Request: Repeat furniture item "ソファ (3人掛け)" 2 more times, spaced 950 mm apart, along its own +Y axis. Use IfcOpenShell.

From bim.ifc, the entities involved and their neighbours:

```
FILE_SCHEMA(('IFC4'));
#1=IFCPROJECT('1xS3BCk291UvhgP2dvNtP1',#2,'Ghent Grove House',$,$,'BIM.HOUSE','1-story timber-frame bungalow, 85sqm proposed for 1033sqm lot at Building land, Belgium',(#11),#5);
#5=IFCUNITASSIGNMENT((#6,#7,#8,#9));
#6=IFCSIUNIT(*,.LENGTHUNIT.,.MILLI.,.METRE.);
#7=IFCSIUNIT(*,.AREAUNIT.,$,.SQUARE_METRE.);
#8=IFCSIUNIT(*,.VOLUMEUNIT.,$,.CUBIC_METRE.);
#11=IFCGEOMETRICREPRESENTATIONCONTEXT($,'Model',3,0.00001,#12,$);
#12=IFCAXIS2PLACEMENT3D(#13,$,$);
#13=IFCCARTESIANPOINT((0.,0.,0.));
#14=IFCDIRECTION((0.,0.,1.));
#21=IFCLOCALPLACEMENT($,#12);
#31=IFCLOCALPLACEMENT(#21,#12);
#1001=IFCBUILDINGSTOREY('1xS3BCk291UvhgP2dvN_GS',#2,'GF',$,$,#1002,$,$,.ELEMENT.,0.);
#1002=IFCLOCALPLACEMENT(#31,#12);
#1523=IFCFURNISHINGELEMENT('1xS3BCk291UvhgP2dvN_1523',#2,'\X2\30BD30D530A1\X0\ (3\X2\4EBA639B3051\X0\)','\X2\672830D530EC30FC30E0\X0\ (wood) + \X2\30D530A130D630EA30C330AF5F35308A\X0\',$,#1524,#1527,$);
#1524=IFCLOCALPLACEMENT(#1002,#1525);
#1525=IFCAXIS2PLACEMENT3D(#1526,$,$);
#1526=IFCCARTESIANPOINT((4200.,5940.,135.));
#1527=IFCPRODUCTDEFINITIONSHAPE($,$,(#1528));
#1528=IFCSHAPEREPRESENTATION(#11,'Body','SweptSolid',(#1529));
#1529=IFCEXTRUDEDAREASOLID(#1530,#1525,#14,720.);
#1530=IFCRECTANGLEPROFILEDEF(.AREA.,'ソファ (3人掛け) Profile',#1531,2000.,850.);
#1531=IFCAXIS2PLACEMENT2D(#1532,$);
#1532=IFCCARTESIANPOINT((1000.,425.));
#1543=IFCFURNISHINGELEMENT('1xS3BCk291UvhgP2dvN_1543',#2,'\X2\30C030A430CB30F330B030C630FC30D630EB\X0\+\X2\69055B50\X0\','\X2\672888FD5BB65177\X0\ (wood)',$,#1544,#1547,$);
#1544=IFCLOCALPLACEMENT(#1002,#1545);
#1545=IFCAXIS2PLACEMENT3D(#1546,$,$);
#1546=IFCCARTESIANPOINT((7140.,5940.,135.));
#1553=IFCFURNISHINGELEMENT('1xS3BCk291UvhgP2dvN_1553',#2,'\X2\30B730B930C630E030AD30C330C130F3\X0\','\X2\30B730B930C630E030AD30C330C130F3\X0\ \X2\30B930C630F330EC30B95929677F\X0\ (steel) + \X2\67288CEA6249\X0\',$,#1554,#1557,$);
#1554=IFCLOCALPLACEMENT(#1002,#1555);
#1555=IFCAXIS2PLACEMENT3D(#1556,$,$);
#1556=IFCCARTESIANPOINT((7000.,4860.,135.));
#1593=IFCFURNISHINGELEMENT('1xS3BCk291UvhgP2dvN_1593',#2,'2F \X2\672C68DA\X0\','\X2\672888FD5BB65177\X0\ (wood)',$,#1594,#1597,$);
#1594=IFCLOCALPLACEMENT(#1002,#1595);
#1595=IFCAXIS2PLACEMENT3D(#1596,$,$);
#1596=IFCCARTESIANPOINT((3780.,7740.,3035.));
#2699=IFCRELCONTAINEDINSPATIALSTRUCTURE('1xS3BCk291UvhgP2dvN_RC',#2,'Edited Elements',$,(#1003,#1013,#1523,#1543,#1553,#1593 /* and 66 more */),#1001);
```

```python
import ifcopenshell
import ifcopenshell.api.geometry
import ifcopenshell.api.root
import ifcopenshell.util.element
import ifcopenshell.util.placement
import ifcopenshell.util.unit

model = ifcopenshell.open("bim.ifc")
unit_scale = ifcopenshell.util.unit.calculate_unit_scale(model)


def reuse_history(source, copy):
    """copy_class also copies each property set's owner history, people and application; keep the originals."""
    for rel in copy.IsDefinedBy:
        if rel.is_a("IfcRelDefinesByProperties") and (history := rel.RelatingPropertyDefinition.OwnerHistory):
            rel.RelatingPropertyDefinition.OwnerHistory = source.OwnerHistory
            ifcopenshell.util.element.remove_deep2(model, history)


source = model.by_guid("1xS3BCk291UvhgP2dvN_1523")
base = ifcopenshell.util.placement.get_local_placement(source.ObjectPlacement)
step = base[:3, 1] * 0.95 / unit_scale

for i in range(1, 3):
    copy = ifcopenshell.api.root.copy_class(model, product=source)
    copy.Representation = ifcopenshell.util.element.copy_deep(
        model, source.Representation, exclude=["IfcGeometricRepresentationContext", "IfcRepresentationMap"]
    )
    reuse_history(source, copy)
    matrix = base.copy()
    matrix[:3, 3] += i * step
    print("added at", matrix[:3, 3].round(3) + 0.0)
    ifcopenshell.api.geometry.edit_object_placement(model, product=copy, matrix=matrix, is_si=False)

model.write("bim-out.ifc")
```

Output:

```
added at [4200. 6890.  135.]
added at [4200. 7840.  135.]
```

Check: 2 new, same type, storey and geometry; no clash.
